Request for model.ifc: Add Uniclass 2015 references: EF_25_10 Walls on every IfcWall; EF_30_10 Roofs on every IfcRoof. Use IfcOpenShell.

First a look at what the model holds.

```python
import ifcopenshell

model = ifcopenshell.open("model.ifc")
print(model.schema)
print("classifications:", [c.Name for c in model.by_type("IfcClassification")])
for ifc_class in ("IfcDoor", "IfcRoof", "IfcStair", "IfcWall", "IfcWindow"):
    print(ifc_class, len(model.by_type(ifc_class)))
```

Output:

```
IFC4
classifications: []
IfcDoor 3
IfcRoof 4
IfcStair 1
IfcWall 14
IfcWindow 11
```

```python
import ifcopenshell
import ifcopenshell.api.classification

model = ifcopenshell.open("model.ifc")

system = ifcopenshell.api.classification.add_classification(model, classification="Uniclass 2015")

codes = {
    "IfcWall": ("EF_25_10", "Walls"),
    "IfcRoof": ("EF_30_10", "Roofs"),
}
for ifc_class, (code, name) in codes.items():
    products = model.by_type(ifc_class)
    ifcopenshell.api.classification.add_reference(
        model, products=products, classification=system, identification=code, name=name
    )
    print(code, len(products))

model.write("model_v2.ifc")
```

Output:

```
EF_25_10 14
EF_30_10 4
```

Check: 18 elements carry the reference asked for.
